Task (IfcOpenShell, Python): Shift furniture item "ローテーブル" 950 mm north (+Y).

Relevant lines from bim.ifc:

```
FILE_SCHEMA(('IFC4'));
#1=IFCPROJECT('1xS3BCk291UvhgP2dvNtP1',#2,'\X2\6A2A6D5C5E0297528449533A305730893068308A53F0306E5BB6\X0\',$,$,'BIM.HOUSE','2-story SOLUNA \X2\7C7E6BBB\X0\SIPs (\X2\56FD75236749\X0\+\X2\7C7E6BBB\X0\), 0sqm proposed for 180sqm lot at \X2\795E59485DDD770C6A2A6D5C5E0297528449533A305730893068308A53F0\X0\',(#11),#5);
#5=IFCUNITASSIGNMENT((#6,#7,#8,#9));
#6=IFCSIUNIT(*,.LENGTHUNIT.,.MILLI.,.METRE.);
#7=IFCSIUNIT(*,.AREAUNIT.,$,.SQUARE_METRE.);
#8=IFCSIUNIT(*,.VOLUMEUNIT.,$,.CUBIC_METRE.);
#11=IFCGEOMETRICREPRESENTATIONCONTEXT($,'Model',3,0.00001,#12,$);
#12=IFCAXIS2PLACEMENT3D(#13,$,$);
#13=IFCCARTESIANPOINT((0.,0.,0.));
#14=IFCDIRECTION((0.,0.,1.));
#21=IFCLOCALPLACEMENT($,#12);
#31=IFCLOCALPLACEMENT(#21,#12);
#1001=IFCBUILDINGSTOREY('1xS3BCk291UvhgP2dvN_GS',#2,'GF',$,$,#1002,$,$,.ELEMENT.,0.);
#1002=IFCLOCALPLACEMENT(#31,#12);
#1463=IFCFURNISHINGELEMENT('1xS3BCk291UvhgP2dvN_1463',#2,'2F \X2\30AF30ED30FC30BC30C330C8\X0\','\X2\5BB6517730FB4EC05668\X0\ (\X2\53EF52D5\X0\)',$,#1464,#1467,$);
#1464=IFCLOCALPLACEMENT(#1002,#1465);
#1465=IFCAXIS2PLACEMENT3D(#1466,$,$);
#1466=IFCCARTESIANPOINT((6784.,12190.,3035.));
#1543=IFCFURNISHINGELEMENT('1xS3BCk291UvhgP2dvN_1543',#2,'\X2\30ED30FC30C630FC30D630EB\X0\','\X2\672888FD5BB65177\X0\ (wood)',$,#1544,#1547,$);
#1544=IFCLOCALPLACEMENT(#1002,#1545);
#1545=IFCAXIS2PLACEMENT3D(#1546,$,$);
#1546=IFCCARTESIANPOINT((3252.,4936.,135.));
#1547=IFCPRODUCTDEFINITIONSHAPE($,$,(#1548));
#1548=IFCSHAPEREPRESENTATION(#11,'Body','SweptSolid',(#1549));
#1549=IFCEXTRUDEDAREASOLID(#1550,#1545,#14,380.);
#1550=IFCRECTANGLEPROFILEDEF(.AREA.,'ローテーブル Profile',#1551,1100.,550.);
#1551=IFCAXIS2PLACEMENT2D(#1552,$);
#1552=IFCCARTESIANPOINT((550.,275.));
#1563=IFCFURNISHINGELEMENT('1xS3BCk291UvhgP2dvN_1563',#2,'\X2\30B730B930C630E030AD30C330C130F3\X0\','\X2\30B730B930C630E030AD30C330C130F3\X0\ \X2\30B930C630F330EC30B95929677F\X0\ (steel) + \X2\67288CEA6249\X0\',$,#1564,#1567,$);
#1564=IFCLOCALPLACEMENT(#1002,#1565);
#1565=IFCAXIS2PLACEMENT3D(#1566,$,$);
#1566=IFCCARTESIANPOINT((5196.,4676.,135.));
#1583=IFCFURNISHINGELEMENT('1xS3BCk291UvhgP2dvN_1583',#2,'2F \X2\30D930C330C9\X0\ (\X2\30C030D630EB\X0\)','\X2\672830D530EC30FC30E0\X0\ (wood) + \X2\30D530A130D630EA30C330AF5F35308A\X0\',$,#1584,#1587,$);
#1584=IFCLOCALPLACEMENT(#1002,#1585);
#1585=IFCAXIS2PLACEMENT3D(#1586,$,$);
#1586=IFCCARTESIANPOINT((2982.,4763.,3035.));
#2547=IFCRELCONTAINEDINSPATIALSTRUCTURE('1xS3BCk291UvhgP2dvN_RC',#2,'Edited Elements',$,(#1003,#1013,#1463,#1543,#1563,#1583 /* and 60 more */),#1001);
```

```python
import ifcopenshell
import ifcopenshell.api.geometry
import ifcopenshell.util.placement
import ifcopenshell.util.unit

model = ifcopenshell.open("bim.ifc")
unit_scale = ifcopenshell.util.unit.calculate_unit_scale(model)

item = model.by_id(1543)
matrix = ifcopenshell.util.placement.get_local_placement(item.ObjectPlacement)
matrix[1, 3] += 0.95 / unit_scale
ifcopenshell.api.geometry.edit_object_placement(model, product=item, matrix=matrix, is_si=False)

print(ifcopenshell.util.placement.get_local_placement(item.ObjectPlacement).round(3) + 0.0)

model.write("bim_updated.ifc")
```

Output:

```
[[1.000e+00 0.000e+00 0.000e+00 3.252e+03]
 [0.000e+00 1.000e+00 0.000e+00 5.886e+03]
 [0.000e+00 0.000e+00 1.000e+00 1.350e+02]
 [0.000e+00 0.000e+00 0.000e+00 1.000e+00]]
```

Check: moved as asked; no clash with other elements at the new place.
